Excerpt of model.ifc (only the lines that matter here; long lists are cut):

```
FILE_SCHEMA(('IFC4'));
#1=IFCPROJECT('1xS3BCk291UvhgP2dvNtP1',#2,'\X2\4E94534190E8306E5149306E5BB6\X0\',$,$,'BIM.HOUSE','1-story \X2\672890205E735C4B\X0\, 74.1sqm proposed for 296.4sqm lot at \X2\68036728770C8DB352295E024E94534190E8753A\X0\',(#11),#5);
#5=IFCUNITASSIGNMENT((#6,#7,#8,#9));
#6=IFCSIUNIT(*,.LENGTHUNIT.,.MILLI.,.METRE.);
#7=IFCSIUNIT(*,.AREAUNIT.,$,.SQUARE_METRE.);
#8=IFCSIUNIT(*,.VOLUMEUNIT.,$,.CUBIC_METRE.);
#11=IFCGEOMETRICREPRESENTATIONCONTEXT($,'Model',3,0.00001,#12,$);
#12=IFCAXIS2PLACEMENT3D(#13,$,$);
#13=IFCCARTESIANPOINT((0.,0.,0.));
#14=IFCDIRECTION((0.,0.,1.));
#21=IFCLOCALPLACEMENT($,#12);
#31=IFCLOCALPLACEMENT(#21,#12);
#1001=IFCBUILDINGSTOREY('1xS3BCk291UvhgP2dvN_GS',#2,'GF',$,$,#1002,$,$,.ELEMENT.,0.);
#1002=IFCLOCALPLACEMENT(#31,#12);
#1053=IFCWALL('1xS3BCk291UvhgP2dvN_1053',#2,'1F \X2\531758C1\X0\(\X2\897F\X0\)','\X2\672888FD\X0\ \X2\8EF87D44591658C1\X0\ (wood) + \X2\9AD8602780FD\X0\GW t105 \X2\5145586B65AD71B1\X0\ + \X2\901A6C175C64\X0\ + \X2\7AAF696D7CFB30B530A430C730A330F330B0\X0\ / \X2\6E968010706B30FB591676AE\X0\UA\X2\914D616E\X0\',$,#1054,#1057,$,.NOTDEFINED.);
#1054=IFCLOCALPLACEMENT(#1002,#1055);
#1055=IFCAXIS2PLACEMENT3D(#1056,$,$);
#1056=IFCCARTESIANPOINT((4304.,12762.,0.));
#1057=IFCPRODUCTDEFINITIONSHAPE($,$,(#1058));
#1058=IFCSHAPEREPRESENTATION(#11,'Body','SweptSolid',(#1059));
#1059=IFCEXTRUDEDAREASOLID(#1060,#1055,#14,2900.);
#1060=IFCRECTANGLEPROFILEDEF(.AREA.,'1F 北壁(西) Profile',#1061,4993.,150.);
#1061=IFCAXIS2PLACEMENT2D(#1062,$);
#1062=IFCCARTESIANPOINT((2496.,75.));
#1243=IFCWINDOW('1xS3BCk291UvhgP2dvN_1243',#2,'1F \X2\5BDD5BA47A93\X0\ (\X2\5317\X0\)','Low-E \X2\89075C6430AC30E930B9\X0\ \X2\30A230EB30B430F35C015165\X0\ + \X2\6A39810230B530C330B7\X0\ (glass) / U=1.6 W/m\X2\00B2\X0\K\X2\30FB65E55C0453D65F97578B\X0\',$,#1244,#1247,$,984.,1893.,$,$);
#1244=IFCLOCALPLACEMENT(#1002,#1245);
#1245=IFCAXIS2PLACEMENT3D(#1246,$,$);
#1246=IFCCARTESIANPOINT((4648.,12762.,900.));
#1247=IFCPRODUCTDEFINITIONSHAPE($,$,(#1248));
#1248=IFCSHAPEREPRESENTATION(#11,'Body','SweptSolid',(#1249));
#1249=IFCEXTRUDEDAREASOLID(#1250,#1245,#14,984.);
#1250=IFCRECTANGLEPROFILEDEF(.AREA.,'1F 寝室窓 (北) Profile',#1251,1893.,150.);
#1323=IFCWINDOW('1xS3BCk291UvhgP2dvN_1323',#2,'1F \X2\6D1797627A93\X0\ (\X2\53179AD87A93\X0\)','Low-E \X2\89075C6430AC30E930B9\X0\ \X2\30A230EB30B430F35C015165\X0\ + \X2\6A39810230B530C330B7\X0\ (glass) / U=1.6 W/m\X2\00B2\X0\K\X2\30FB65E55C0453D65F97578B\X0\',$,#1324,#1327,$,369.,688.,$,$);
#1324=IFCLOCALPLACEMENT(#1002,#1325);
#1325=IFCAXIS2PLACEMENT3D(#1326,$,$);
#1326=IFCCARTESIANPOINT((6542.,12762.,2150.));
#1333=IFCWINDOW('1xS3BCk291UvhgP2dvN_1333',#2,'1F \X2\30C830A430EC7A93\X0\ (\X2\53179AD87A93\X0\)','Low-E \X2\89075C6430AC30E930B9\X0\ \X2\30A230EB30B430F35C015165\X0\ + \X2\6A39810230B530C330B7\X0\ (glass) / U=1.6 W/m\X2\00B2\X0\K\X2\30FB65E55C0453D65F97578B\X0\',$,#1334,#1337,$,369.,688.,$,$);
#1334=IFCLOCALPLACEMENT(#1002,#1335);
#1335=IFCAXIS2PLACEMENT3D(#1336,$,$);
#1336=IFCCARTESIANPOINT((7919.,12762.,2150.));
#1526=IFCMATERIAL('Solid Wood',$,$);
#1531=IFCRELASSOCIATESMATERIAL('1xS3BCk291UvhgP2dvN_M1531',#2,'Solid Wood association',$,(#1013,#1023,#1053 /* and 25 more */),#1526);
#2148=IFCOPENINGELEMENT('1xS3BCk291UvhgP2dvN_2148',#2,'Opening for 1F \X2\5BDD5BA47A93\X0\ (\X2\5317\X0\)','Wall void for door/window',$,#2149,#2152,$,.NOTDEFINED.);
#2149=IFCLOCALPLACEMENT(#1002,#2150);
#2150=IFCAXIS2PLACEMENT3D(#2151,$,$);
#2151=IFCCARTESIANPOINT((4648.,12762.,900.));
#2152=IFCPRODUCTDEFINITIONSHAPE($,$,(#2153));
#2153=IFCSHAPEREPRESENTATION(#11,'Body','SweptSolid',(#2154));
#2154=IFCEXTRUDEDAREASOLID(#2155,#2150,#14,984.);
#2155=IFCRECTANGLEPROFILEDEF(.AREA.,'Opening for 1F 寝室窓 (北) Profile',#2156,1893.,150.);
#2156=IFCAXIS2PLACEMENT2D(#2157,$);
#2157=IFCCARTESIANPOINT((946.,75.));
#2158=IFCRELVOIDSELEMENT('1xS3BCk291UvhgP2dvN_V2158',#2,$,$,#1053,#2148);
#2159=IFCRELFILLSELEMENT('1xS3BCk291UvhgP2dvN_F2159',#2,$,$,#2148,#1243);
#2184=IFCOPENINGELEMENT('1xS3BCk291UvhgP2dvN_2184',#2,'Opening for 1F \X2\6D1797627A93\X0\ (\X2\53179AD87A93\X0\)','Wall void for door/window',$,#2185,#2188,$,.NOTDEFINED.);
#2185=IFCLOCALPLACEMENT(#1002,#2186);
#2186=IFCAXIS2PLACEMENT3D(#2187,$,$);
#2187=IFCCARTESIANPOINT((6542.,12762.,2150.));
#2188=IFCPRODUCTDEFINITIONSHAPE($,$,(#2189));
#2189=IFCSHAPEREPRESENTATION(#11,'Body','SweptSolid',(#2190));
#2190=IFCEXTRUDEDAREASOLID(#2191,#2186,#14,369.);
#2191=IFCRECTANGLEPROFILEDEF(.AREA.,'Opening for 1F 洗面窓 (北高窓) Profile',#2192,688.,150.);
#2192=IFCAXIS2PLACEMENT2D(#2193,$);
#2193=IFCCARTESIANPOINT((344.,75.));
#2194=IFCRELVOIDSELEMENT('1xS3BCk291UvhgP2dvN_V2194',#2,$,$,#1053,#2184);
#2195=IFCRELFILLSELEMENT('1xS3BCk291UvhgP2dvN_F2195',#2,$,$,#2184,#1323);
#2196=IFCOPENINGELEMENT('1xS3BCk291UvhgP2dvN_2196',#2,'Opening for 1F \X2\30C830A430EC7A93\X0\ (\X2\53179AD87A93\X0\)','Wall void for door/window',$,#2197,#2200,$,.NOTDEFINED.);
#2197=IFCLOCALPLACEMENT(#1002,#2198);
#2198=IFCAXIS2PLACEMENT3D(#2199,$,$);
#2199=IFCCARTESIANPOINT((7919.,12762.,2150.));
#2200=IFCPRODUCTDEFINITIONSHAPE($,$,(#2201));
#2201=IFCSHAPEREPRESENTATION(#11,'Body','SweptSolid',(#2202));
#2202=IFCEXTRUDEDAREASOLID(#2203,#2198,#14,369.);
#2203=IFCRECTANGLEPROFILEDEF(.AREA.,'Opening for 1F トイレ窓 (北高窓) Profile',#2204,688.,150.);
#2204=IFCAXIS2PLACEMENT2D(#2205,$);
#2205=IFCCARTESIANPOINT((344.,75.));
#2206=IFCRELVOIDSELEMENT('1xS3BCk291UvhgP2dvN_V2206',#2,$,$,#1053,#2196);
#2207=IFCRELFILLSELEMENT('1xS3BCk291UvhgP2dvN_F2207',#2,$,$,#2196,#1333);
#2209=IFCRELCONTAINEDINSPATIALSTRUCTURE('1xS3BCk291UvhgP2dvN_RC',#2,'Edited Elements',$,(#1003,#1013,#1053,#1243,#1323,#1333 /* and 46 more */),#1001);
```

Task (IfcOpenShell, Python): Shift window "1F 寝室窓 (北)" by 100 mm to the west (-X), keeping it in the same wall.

```python
import ifcopenshell
import ifcopenshell.api.geometry
import ifcopenshell.util.placement
import ifcopenshell.util.unit

model = ifcopenshell.open("model.ifc")
unit_scale = ifcopenshell.util.unit.calculate_unit_scale(model)

window = model.by_guid("1xS3BCk291UvhgP2dvN_1243")
opening = window.FillsVoids[0].RelatingOpeningElement
wall = opening.VoidsElements[0].RelatingBuildingElement

wall_matrix = ifcopenshell.util.placement.get_local_placement(wall.ObjectPlacement)
shift = wall_matrix[:3, 0] * -0.1 / unit_scale
before = ifcopenshell.util.placement.get_local_placement(window.ObjectPlacement)[:3, 3].copy()

# The window is not placed relative to its opening, so move both.
for product in (opening, window):
    matrix = ifcopenshell.util.placement.get_local_placement(product.ObjectPlacement)
    matrix[:3, 3] += shift
    ifcopenshell.api.geometry.edit_object_placement(model, product=product, matrix=matrix, is_si=False)

after = ifcopenshell.util.placement.get_local_placement(window.ObjectPlacement)[:3, 3]
print("window moved by", (after - before).round(3) + 0.0)

model.write("model_updated.ifc")
```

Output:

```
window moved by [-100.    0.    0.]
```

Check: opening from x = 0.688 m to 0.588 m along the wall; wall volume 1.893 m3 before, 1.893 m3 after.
